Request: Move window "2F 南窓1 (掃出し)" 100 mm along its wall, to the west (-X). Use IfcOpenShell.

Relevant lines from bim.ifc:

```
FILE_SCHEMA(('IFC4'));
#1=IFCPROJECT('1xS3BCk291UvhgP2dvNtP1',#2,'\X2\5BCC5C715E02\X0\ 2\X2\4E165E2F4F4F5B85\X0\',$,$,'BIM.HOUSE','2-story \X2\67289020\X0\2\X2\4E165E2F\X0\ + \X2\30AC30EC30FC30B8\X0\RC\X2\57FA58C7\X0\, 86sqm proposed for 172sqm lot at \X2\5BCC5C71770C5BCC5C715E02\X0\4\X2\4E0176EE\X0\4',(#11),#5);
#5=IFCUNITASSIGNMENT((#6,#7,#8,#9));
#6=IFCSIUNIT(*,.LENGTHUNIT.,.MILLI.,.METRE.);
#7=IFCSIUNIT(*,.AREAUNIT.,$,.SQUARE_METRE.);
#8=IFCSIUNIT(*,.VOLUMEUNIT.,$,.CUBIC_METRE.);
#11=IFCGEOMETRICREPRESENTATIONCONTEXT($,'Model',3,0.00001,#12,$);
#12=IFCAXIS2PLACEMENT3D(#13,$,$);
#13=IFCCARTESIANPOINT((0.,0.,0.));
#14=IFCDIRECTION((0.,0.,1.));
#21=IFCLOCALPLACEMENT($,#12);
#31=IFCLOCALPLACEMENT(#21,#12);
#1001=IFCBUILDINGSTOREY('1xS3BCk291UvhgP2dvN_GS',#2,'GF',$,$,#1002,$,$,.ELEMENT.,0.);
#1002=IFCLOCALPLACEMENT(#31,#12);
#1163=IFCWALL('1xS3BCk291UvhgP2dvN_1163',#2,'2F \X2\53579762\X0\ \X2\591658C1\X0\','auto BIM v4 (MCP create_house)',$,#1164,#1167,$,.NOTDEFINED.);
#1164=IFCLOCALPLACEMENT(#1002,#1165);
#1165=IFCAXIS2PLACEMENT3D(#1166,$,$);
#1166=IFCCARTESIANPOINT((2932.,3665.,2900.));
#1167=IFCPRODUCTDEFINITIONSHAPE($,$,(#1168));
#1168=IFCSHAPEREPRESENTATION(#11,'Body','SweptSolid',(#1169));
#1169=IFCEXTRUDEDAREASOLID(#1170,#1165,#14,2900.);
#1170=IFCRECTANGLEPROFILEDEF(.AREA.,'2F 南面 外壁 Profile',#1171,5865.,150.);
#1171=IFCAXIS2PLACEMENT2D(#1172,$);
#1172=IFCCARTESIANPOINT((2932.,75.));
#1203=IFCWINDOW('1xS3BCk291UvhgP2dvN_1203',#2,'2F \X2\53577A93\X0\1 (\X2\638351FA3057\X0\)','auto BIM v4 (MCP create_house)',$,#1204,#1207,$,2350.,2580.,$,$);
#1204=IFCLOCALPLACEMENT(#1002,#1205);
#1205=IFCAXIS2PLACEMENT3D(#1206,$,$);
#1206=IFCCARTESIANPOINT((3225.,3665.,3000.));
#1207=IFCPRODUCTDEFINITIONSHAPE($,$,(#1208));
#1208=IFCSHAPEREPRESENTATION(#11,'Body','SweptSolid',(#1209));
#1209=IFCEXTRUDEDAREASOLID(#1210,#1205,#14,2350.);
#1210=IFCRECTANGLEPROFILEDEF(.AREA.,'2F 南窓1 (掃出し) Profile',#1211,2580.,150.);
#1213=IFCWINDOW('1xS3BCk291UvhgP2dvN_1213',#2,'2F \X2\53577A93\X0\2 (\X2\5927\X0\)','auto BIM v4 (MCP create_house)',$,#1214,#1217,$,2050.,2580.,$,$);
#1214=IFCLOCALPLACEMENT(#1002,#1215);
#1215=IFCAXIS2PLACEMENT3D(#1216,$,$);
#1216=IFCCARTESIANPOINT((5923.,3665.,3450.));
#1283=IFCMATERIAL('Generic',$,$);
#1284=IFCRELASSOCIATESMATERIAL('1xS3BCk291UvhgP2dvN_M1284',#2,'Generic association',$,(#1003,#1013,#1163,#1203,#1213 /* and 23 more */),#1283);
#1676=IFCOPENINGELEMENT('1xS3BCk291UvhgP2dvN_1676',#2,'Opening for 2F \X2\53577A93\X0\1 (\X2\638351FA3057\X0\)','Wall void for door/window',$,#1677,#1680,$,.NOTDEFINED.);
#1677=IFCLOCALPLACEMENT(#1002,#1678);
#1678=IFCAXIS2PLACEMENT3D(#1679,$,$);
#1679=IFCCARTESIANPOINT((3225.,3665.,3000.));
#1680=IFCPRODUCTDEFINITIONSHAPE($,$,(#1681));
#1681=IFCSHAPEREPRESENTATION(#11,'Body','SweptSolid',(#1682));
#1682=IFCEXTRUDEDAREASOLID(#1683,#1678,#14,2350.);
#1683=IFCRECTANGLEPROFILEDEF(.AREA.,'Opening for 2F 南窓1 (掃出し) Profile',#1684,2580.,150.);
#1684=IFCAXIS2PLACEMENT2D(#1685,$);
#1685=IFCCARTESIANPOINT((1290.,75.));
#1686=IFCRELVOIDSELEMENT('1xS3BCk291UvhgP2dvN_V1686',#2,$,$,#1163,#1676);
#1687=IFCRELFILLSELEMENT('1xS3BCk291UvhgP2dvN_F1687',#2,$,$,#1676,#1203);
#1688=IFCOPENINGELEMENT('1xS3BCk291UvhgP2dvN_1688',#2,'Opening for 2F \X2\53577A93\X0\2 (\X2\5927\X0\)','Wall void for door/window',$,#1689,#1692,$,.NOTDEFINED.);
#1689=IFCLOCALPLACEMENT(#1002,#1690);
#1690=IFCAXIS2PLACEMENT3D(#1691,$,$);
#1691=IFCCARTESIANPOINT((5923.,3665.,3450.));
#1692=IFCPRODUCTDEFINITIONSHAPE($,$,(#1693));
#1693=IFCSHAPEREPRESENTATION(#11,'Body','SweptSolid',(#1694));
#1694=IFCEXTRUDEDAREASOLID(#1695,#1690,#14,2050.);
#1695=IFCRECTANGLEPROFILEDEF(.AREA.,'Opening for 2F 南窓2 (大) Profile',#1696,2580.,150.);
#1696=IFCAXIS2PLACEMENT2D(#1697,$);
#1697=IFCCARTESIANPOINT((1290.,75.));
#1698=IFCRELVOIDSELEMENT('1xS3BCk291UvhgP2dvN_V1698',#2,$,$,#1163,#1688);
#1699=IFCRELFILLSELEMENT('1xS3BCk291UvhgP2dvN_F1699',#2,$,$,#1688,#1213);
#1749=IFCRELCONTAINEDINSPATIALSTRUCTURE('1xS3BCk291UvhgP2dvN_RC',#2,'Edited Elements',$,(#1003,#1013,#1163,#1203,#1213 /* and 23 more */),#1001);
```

```python
import ifcopenshell
import ifcopenshell.api.geometry
import ifcopenshell.util.placement
import ifcopenshell.util.unit

model = ifcopenshell.open("bim.ifc")
unit_scale = ifcopenshell.util.unit.calculate_unit_scale(model)

window = model.by_id(1203)
opening = window.FillsVoids[0].RelatingOpeningElement
wall = opening.VoidsElements[0].RelatingBuildingElement

wall_matrix = ifcopenshell.util.placement.get_local_placement(wall.ObjectPlacement)
shift = wall_matrix[:3, 0] * -0.1 / unit_scale
before = ifcopenshell.util.placement.get_local_placement(window.ObjectPlacement)[:3, 3].copy()

# The window is not placed relative to its opening, so move both.
for product in (opening, window):
    matrix = ifcopenshell.util.placement.get_local_placement(product.ObjectPlacement)
    matrix[:3, 3] += shift
    ifcopenshell.api.geometry.edit_object_placement(model, product=product, matrix=matrix, is_si=False)

after = ifcopenshell.util.placement.get_local_placement(window.ObjectPlacement)[:3, 3]
print("window moved by", (after - before).round(3) + 0.0)

model.write("bim_edited.ifc")
```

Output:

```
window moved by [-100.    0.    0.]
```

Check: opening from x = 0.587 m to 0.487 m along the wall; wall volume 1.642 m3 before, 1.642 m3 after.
